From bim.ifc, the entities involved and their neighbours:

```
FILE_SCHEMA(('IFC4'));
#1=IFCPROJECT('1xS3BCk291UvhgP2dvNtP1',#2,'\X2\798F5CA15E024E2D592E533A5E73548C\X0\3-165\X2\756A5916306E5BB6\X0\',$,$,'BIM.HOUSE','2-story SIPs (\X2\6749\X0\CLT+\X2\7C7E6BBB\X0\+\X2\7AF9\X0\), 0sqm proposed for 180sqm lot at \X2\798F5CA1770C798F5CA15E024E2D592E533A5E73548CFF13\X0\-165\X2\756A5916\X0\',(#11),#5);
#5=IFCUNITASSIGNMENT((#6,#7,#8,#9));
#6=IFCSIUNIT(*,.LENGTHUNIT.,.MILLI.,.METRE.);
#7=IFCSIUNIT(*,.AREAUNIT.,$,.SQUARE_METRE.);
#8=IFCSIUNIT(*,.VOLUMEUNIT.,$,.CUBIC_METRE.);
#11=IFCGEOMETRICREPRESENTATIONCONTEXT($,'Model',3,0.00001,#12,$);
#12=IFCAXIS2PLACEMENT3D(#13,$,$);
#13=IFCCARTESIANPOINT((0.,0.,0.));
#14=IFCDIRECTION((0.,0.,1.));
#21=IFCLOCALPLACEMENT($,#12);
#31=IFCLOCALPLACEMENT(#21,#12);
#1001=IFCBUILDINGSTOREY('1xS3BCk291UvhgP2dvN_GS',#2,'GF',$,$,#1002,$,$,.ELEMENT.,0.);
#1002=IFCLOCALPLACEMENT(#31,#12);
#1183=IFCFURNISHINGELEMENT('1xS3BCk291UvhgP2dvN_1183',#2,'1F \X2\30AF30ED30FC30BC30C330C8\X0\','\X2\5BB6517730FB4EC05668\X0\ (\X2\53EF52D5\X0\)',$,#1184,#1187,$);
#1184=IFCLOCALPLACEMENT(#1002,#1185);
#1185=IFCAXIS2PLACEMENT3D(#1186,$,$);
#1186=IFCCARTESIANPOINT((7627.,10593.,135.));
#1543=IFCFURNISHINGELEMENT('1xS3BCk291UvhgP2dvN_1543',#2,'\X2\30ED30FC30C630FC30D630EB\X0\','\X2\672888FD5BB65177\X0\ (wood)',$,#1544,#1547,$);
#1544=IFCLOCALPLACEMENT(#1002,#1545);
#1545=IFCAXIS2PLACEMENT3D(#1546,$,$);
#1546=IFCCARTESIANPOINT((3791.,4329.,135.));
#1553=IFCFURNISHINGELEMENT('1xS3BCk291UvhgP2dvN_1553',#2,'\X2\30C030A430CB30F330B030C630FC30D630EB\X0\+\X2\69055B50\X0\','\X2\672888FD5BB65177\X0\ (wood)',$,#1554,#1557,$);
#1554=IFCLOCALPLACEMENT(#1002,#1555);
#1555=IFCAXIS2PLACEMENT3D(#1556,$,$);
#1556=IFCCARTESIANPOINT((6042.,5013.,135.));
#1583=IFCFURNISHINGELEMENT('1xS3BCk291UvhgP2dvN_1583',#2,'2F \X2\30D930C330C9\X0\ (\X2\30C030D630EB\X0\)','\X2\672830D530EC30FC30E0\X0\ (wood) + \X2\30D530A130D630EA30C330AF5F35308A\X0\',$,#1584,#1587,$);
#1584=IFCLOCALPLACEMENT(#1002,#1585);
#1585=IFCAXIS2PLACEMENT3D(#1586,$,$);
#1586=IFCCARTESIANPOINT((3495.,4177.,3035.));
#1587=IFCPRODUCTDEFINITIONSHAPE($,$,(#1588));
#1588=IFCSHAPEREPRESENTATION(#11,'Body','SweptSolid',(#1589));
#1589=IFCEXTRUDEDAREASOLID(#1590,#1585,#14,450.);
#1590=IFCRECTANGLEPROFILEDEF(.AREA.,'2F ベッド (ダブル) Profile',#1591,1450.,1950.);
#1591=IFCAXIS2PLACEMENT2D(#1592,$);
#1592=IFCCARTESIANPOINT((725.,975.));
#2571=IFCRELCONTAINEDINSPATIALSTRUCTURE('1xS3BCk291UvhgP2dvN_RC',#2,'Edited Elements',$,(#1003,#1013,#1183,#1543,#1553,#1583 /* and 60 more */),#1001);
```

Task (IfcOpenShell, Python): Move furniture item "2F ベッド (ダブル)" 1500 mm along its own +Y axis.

```python
import ifcopenshell
import ifcopenshell.api.geometry
import ifcopenshell.util.placement
import ifcopenshell.util.unit

model = ifcopenshell.open("bim.ifc")
unit_scale = ifcopenshell.util.unit.calculate_unit_scale(model)

item = model.by_guid("1xS3BCk291UvhgP2dvN_1583")
matrix = ifcopenshell.util.placement.get_local_placement(item.ObjectPlacement)
matrix[:3, 3] += matrix[:3, 1] * 1.5 / unit_scale
ifcopenshell.api.geometry.edit_object_placement(model, product=item, matrix=matrix, is_si=False)

print(ifcopenshell.util.placement.get_local_placement(item.ObjectPlacement).round(3) + 0.0)

model.write("bim_rev.ifc")
```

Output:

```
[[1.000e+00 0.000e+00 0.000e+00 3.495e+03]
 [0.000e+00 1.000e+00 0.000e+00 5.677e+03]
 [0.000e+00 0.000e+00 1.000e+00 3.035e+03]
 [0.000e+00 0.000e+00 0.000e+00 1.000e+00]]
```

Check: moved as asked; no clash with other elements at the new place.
